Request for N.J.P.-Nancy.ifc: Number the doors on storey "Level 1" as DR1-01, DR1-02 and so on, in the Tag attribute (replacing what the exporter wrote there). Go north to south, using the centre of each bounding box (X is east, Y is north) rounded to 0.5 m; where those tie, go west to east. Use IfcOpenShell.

First a look at what the model holds.

```python
import ifcopenshell
import ifcopenshell.util.element
import ifcopenshell.util.placement

model = ifcopenshell.open("N.J.P.-Nancy.ifc")
print(model.schema)
storey = next(s for s in model.by_type("IfcBuildingStorey") if s.Name == "Level 1")
doors = [e for e in ifcopenshell.util.element.get_decomposition(storey) if e.is_a("IfcDoor")]
for e in sorted(doors, key=lambda e: e.id()):
    origin = ifcopenshell.util.placement.get_local_placement(e.ObjectPlacement)[:3, 3]
    print(e.id(), e.Tag, e.Name, origin.round(2) + 0.0, sep=" | ")
```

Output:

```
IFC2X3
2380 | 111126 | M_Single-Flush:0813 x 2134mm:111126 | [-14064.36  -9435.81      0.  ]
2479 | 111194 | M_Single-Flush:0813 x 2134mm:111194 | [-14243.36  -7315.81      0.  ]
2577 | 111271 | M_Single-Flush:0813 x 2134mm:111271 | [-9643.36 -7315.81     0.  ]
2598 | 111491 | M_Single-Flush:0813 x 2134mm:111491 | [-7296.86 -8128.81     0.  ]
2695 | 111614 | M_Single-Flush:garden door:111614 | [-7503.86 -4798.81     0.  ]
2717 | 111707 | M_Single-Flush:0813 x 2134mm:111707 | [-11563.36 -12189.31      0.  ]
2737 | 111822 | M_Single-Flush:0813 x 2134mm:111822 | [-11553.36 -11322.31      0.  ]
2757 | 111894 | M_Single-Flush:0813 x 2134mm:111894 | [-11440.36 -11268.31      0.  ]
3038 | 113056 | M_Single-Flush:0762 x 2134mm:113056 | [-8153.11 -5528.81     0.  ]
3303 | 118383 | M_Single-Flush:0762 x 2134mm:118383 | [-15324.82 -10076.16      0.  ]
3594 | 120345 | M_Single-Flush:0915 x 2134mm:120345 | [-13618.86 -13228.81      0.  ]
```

```python
import ifcopenshell
import ifcopenshell.geom
import ifcopenshell.util.element
import ifcopenshell.util.shape

model = ifcopenshell.open("N.J.P.-Nancy.ifc")
settings = ifcopenshell.geom.settings()
settings.set("use-world-coords", True)


def centre(element):
    shape = ifcopenshell.geom.create_shape(settings, element)
    return ifcopenshell.util.shape.get_bbox_centroid(shape.geometry)


storey = next(s for s in model.by_type("IfcBuildingStorey") if s.Name == "Level 1")
doors = [e for e in ifcopenshell.util.element.get_decomposition(storey) if e.is_a("IfcDoor")]

# Insertion points can sit at a corner or the storey origin, so sort by the geometry (in metres).
centres = {e: centre(e) for e in doors}
doors.sort(key=lambda e: (-round(centres[e][1] / 0.5), centres[e][0]))

for i, e in enumerate(doors, start=1):
    number = f"DR1-{i:02d}"
    e.Tag = number
    print(e.id(), number)

model.write("N.J.P.-Nancy_updated.ifc")
```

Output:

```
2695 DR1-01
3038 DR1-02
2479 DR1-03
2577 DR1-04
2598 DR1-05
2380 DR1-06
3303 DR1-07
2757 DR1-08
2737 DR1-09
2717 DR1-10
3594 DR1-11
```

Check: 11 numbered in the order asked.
